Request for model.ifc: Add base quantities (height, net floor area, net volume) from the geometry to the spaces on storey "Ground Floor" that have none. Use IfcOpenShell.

First a look at what the model holds.

```python
import ifcopenshell
import ifcopenshell.util.element
import ifcopenshell.util.unit

model = ifcopenshell.open("model.ifc")
print(model.schema)
for unit_type in ("LENGTHUNIT", "AREAUNIT", "VOLUMEUNIT"):
    print(unit_type, ifcopenshell.util.unit.calculate_unit_scale(model, unit_type))
storey = next(s for s in model.by_type("IfcBuildingStorey") if s.Name == "Ground Floor")
spaces = [e for e in ifcopenshell.util.element.get_decomposition(storey) if e.is_a("IfcSpace")]
for e in sorted(spaces, key=lambda e: e.id()):
    print(e.id(), e.is_a(), e.Name, list(ifcopenshell.util.element.get_psets(e, qtos_only=True)), sep=" | ")
```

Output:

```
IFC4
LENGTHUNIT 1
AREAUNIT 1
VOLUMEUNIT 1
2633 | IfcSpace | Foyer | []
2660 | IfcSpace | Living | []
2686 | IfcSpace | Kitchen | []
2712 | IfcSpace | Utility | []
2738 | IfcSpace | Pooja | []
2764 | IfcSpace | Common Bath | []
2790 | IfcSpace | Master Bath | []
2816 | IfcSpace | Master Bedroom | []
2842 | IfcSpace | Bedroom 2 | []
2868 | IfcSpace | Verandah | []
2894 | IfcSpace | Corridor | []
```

```python
import ifcopenshell
import ifcopenshell.api.pset
import ifcopenshell.geom
import ifcopenshell.util.element
import ifcopenshell.util.shape
import ifcopenshell.util.unit

model = ifcopenshell.open("model.ifc")
unit_scale = ifcopenshell.util.unit.calculate_unit_scale(model)
area_scale = ifcopenshell.util.unit.calculate_unit_scale(model, "AREAUNIT")
volume_scale = ifcopenshell.util.unit.calculate_unit_scale(model, "VOLUMEUNIT")
settings = ifcopenshell.geom.settings()

storey = next(s for s in model.by_type("IfcBuildingStorey") if s.Name == "Ground Floor")
spaces = [e for e in ifcopenshell.util.element.get_decomposition(storey) if e.is_a("IfcSpace")]

for e in sorted(spaces, key=lambda e: e.id()):
    if ifcopenshell.util.element.get_psets(e, qtos_only=True, should_inherit=False):
        continue
    # Geometry comes back in metres, in the element's own axes.
    shape = ifcopenshell.geom.create_shape(settings, e)
    values = {
        "Height": ifcopenshell.util.shape.get_z(shape.geometry) / unit_scale,
        "NetFloorArea": ifcopenshell.util.shape.get_footprint_area(shape.geometry) / area_scale,
        "NetVolume": ifcopenshell.util.shape.get_volume(shape.geometry) / volume_scale,
    }
    qto = ifcopenshell.api.pset.add_qto(model, product=e, name="Qto_SpaceBaseQuantities")
    ifcopenshell.api.pset.edit_qto(model, qto=qto, properties=values)
    print(e.id(), {k: round(v, 3) for k, v in values.items()})

model.write("model_updated.ifc")
```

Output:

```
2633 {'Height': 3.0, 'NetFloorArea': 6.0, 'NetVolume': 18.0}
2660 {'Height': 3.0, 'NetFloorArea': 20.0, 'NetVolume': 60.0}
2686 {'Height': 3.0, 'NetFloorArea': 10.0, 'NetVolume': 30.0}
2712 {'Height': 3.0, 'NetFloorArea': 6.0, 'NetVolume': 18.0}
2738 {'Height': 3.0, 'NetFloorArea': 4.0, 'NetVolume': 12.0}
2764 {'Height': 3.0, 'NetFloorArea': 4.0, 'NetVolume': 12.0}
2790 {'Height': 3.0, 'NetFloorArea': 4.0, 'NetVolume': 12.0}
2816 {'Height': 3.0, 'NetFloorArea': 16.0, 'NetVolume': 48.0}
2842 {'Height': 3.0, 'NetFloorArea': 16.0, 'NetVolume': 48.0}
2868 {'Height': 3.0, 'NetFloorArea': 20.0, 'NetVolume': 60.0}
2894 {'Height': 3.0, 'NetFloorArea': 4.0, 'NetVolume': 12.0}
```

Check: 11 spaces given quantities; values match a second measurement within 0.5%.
